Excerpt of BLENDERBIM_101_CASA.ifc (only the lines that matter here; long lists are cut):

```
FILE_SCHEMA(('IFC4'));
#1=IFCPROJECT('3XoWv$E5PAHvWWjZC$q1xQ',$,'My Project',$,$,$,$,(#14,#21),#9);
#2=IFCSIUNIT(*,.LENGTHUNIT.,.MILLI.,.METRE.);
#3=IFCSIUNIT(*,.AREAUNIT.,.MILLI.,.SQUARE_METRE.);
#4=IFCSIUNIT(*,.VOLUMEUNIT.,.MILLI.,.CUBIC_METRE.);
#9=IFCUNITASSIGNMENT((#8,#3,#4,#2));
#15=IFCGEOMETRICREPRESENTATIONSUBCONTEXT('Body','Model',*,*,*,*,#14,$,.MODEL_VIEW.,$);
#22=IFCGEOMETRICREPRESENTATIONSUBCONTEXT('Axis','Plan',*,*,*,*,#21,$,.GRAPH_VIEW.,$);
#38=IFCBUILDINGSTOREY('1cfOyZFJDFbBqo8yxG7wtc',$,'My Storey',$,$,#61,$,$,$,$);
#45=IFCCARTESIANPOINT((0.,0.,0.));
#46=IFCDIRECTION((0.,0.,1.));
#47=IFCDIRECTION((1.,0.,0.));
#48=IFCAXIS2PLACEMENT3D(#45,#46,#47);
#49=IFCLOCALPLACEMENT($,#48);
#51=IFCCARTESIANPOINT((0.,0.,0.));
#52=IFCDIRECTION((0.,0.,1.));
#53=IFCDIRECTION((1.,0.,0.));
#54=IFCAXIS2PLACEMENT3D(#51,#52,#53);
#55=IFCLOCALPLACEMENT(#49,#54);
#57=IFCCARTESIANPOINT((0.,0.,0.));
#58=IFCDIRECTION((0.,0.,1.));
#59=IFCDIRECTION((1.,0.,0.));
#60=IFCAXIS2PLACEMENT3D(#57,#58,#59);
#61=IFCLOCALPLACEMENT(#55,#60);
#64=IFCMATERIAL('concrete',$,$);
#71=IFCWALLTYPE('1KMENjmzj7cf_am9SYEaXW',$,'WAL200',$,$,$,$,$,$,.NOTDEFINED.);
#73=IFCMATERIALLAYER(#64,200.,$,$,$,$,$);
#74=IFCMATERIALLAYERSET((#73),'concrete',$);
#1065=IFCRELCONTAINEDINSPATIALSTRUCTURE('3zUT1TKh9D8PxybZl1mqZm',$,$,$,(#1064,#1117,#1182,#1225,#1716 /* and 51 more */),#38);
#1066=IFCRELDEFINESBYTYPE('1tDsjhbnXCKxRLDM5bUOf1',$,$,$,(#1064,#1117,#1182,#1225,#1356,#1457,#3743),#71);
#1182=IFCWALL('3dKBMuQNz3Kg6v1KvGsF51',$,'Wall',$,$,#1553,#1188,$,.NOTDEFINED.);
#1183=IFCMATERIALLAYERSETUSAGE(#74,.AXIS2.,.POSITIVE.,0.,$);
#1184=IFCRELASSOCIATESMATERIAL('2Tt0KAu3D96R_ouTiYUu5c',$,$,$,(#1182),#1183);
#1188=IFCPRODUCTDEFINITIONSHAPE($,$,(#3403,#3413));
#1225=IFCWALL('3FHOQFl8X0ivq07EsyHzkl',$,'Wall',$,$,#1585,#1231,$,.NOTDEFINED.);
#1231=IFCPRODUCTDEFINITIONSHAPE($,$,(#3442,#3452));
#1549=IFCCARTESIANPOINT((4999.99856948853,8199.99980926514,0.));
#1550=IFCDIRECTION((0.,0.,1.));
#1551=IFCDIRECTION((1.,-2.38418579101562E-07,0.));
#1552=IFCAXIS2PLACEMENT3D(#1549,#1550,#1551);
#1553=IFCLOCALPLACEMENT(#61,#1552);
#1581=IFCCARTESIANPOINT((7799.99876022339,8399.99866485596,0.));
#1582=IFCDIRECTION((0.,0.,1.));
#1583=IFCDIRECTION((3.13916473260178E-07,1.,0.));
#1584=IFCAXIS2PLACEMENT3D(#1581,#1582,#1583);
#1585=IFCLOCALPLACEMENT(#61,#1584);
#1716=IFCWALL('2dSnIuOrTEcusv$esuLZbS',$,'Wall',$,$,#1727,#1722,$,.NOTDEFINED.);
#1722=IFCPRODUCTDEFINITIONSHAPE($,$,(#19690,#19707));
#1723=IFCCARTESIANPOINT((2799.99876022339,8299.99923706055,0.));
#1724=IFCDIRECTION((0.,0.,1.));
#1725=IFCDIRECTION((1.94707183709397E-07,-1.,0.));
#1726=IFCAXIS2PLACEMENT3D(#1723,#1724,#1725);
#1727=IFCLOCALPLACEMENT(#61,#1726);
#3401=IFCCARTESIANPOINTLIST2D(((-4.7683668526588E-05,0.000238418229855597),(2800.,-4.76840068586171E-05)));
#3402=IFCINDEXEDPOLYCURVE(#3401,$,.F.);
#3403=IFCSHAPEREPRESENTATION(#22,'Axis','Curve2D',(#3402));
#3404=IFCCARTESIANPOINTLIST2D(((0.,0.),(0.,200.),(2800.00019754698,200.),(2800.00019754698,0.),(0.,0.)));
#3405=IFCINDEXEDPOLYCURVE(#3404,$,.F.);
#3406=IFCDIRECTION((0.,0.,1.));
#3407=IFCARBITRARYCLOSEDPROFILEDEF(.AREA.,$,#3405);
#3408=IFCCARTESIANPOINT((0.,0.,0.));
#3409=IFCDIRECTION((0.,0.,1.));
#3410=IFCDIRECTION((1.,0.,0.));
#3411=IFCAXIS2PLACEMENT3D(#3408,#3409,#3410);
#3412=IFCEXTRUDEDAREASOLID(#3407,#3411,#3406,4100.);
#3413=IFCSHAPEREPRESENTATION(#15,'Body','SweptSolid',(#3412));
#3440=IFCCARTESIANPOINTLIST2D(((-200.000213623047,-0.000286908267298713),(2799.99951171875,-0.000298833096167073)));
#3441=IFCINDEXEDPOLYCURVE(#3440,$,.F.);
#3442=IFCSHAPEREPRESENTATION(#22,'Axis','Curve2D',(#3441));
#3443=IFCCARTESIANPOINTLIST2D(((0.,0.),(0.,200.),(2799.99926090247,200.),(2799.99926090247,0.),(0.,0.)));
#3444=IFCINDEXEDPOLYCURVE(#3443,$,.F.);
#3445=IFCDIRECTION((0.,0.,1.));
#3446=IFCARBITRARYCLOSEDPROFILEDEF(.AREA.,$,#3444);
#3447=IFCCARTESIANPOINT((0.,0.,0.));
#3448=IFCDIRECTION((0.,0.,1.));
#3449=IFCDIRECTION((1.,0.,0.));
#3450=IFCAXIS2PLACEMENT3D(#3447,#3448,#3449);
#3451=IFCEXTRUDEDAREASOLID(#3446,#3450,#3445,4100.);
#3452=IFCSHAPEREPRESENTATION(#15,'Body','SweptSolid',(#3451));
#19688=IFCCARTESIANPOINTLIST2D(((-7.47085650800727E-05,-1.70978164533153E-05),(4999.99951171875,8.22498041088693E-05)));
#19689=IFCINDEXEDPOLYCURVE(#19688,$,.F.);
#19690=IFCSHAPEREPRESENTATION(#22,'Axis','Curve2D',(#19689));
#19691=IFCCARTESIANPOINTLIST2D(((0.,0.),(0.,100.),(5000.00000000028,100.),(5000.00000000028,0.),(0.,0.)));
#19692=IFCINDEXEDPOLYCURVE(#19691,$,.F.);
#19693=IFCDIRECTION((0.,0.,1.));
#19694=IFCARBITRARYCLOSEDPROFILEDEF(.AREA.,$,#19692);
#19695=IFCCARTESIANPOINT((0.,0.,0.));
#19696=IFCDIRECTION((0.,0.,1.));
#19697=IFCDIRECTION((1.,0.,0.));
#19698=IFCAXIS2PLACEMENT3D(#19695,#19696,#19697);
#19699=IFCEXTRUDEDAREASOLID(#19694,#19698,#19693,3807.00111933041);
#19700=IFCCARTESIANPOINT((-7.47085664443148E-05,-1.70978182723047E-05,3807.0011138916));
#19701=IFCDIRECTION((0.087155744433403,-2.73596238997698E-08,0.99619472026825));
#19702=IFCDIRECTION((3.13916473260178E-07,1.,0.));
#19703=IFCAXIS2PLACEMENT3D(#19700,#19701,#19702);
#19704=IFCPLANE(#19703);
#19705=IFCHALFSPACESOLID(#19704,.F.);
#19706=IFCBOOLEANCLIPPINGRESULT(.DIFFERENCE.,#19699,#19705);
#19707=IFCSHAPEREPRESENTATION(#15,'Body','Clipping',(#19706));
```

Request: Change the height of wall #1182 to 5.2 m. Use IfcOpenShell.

```python
import ifcopenshell
import ifcopenshell.geom
import ifcopenshell.util.representation
import ifcopenshell.util.shape
import ifcopenshell.util.unit

model = ifcopenshell.open("BLENDERBIM_101_CASA.ifc")
unit_scale = ifcopenshell.util.unit.calculate_unit_scale(model)
settings = ifcopenshell.geom.settings()


def volume(element):
    """Net volume in cubic metres, openings subtracted."""
    shape = ifcopenshell.geom.create_shape(settings, element)
    return ifcopenshell.util.shape.get_volume(shape.geometry)


wall = model.by_id(1182)
before = volume(wall)

body = ifcopenshell.util.representation.get_representation(wall, "Model", "Body")
solid = body.Items[0]
old_height = solid.Depth
solid.Depth = 5.2 / unit_scale
after = volume(wall)

print(f"height {old_height:g} -> {solid.Depth:g}, volume {before:.3f} -> {after:.3f} m3")

model.write("BLENDERBIM_101_CASA-out.ifc")
```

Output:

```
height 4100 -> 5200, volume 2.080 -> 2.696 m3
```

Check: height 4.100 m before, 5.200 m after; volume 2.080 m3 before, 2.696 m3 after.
